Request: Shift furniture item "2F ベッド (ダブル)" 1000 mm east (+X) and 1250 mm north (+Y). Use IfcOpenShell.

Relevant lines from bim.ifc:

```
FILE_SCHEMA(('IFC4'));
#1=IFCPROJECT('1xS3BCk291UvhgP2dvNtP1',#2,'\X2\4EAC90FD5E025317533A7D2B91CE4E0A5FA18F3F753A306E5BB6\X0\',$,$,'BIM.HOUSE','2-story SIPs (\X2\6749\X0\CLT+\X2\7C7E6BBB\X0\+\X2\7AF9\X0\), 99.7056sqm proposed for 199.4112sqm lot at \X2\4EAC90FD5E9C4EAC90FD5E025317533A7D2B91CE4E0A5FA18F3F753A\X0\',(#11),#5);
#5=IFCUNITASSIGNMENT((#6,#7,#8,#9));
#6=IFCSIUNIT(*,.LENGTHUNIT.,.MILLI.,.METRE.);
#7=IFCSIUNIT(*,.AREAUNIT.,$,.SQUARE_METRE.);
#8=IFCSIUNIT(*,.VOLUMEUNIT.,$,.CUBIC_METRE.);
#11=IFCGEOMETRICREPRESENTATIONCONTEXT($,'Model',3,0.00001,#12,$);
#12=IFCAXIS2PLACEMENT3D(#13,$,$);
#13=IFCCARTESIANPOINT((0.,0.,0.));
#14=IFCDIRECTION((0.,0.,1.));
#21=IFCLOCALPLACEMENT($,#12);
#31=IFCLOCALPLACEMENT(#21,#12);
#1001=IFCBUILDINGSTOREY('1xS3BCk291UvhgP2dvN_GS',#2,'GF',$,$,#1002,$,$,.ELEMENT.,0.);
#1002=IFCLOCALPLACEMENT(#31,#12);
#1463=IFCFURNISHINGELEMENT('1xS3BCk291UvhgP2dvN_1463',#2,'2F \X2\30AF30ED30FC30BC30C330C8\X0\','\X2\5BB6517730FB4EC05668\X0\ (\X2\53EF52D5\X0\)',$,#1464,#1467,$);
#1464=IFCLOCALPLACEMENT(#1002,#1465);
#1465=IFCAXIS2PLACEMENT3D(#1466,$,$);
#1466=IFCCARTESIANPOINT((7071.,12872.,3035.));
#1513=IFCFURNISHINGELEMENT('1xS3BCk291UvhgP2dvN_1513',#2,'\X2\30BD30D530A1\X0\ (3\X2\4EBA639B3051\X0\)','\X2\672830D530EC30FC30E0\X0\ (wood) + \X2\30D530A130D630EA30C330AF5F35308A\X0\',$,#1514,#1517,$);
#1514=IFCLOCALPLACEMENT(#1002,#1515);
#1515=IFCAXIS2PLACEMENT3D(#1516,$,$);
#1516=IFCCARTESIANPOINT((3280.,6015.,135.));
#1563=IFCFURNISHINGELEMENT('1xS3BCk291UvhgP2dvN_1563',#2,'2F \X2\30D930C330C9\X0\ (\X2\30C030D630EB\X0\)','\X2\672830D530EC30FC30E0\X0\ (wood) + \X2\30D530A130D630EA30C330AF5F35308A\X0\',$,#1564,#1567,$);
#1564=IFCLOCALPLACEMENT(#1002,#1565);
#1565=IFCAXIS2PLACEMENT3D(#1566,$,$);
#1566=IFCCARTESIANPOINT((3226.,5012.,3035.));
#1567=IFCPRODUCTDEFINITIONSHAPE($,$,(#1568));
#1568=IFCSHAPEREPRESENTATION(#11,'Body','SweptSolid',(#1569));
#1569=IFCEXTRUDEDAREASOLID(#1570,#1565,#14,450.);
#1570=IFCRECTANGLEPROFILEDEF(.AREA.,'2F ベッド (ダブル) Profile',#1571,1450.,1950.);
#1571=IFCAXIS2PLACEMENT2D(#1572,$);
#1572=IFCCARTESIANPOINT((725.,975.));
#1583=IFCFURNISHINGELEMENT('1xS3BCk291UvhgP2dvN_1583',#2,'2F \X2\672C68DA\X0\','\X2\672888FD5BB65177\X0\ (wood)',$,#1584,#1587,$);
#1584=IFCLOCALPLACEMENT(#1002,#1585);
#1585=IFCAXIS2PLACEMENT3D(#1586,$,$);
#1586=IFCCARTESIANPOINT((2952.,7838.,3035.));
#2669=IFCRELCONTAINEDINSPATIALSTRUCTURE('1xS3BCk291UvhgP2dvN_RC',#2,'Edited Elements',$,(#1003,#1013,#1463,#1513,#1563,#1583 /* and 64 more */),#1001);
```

```python
import ifcopenshell
import ifcopenshell.api.geometry
import ifcopenshell.util.placement

model = ifcopenshell.open("bim.ifc")

item = model.by_id(1563)
matrix = ifcopenshell.util.placement.get_local_placement(item.ObjectPlacement)
matrix[0, 3] += 1000.0
matrix[1, 3] += 1250.0
ifcopenshell.api.geometry.edit_object_placement(model, product=item, matrix=matrix, is_si=False)

print(ifcopenshell.util.placement.get_local_placement(item.ObjectPlacement).round(3) + 0.0)

model.write("bim_rev.ifc")
```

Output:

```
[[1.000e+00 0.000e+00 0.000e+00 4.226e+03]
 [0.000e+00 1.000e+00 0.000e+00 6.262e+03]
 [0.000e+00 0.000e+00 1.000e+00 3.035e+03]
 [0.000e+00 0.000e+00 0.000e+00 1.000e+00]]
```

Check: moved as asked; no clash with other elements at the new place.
